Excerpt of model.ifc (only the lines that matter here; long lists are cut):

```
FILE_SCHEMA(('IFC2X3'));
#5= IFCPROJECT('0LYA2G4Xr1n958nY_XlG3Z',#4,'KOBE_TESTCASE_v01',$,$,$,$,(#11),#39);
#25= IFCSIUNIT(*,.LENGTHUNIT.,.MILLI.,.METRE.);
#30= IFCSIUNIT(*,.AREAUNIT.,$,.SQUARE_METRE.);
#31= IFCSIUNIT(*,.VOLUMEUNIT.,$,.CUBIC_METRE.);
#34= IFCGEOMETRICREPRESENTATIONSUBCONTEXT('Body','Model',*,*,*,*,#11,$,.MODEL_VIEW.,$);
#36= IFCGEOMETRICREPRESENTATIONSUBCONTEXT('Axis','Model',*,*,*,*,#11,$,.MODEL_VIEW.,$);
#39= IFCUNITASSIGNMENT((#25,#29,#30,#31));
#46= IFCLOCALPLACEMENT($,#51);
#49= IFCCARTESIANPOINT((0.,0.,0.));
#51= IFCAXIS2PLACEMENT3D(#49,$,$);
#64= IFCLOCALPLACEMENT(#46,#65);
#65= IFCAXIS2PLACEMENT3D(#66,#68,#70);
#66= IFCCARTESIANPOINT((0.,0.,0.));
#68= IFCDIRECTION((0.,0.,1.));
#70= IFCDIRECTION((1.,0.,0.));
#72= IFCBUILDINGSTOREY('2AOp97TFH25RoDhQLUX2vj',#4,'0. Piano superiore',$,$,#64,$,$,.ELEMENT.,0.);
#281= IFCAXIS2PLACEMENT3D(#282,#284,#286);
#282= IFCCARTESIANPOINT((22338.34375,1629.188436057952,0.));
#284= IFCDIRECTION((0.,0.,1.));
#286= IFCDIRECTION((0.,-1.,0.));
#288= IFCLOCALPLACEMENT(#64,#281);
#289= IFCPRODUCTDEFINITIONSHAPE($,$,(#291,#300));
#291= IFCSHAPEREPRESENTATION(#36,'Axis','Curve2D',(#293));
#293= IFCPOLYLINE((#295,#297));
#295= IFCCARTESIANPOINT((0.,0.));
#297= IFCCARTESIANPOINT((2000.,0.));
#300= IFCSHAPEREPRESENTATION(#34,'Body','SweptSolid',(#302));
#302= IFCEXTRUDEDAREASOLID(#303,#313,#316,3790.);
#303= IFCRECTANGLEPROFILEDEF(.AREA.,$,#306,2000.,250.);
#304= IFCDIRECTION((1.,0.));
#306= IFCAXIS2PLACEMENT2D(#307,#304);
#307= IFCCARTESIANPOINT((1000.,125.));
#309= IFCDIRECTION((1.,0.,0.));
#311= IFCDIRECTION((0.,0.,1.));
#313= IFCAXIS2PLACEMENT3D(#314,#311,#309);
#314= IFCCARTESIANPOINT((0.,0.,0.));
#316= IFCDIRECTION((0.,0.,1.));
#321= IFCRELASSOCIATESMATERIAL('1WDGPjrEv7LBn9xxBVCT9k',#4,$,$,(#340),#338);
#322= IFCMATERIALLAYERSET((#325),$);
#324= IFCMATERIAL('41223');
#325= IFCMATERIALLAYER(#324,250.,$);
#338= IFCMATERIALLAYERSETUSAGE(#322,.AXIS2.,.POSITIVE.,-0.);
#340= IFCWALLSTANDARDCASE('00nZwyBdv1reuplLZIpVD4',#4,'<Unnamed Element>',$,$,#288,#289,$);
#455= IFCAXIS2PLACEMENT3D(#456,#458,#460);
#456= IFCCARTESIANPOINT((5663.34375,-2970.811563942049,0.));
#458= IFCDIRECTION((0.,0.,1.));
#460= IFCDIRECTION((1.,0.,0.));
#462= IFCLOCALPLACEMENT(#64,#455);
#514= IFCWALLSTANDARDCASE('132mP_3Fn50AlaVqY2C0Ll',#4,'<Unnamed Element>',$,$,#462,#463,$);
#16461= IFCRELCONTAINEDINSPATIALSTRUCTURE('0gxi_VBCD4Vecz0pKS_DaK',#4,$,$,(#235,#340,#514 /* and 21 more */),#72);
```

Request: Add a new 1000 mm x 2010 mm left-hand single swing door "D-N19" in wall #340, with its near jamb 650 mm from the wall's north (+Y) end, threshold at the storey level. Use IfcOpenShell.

```python
import numpy as np
import ifcopenshell
import ifcopenshell.api.feature
import ifcopenshell.api.geometry
import ifcopenshell.api.root
import ifcopenshell.api.spatial
import ifcopenshell.api.type
import ifcopenshell.geom
import ifcopenshell.util.element
import ifcopenshell.util.placement
import ifcopenshell.util.representation
import ifcopenshell.util.shape
import ifcopenshell.util.unit

model = ifcopenshell.open("model.ifc")
unit_scale = ifcopenshell.util.unit.calculate_unit_scale(model)
settings = ifcopenshell.geom.settings()


def volume(element):
    """Net volume in cubic metres, openings subtracted."""
    shape = ifcopenshell.geom.create_shape(settings, element)
    return ifcopenshell.util.shape.get_volume(shape.geometry)


wall = model.by_guid("00nZwyBdv1reuplLZIpVD4")
storey = ifcopenshell.util.element.get_container(wall, ifc_class="IfcBuildingStorey")
context = ifcopenshell.util.representation.get_context(model, "Model", "Body", "MODEL_VIEW")
before = volume(wall)

width, height, from_end, sill = 1, 2.01, 0.65, 0.0  # metres

# The wall runs along its own X axis, and the end named is its -X end.
wall_shape = ifcopenshell.geom.create_shape(settings, wall)
x, y, z = ifcopenshell.util.shape.get_vertices(wall_shape.geometry).T
start = x.min() + from_end
face, thickness = float(y.min()), float(y.max() - y.min())
wall_matrix = ifcopenshell.util.placement.get_local_placement(wall.ObjectPlacement)
level = ifcopenshell.util.placement.get_local_placement(storey.ObjectPlacement)[2, 3]


def in_wall(x, y):
    """Placement at x, y metres in the wall's axes, at sill height."""
    matrix = wall_matrix.copy()
    matrix[:, 3] = wall_matrix @ np.array([x / unit_scale, y / unit_scale, 0.0, 1.0])
    matrix[2, 3] = level + sill / unit_scale
    return matrix


# Opening: a box that overshoots both wall faces by 50 mm.
opening = ifcopenshell.api.root.create_entity(model, ifc_class="IfcOpeningElement")
box = ifcopenshell.api.geometry.add_wall_representation(
    model, context=context, length=width, height=height, thickness=thickness + 0.1
)
ifcopenshell.api.geometry.assign_representation(model, product=opening, representation=box)
ifcopenshell.api.geometry.edit_object_placement(model, product=opening, matrix=in_wall(start, face - 0.05), is_si=False)
ifcopenshell.api.feature.add_feature(model, feature=opening, element=wall)

door = ifcopenshell.api.root.create_entity(model, ifc_class="IfcDoor", name="D-N19")
door.OverallWidth, door.OverallHeight = width / unit_scale, height / unit_scale
body = ifcopenshell.api.geometry.add_door_representation(
    model,
    context=context,
    overall_width=door.OverallWidth,
    overall_height=door.OverallHeight,
    operation_type="SINGLE_SWING_LEFT",
    lining_properties={"LiningDepth": thickness / unit_scale, "ThresholdDepth": thickness / unit_scale},
)
ifcopenshell.api.geometry.assign_representation(model, product=door, representation=body)
ifcopenshell.api.spatial.assign_container(model, products=[door], relating_structure=storey)
fills = ifcopenshell.api.feature.add_filling(model, opening=opening, element=door)
fills.OwnerHistory = door.OwnerHistory  # required in IFC2X3

# IFC2X3 keeps the operation on the door style.
style = ifcopenshell.api.root.create_entity(model, ifc_class="IfcDoorStyle", name="D-N19")
style.OperationType, style.ConstructionType = "SINGLE_SWING_LEFT", "NOTDEFINED"
style.ParameterTakesPrecedence = style.Sizeable = False
ifcopenshell.api.type.assign_type(model, related_objects=[door], relating_type=style)

# The lining spans the wall, so the door starts at the wall face.
ifcopenshell.api.geometry.edit_object_placement(model, product=door, matrix=in_wall(start, face), is_si=False)

after = volume(wall)

print(f"wall volume {before:.3f} -> {after:.3f} m3")

model.write("model_edited.ifc")
```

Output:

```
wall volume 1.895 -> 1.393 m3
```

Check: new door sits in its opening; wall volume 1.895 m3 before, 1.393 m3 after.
